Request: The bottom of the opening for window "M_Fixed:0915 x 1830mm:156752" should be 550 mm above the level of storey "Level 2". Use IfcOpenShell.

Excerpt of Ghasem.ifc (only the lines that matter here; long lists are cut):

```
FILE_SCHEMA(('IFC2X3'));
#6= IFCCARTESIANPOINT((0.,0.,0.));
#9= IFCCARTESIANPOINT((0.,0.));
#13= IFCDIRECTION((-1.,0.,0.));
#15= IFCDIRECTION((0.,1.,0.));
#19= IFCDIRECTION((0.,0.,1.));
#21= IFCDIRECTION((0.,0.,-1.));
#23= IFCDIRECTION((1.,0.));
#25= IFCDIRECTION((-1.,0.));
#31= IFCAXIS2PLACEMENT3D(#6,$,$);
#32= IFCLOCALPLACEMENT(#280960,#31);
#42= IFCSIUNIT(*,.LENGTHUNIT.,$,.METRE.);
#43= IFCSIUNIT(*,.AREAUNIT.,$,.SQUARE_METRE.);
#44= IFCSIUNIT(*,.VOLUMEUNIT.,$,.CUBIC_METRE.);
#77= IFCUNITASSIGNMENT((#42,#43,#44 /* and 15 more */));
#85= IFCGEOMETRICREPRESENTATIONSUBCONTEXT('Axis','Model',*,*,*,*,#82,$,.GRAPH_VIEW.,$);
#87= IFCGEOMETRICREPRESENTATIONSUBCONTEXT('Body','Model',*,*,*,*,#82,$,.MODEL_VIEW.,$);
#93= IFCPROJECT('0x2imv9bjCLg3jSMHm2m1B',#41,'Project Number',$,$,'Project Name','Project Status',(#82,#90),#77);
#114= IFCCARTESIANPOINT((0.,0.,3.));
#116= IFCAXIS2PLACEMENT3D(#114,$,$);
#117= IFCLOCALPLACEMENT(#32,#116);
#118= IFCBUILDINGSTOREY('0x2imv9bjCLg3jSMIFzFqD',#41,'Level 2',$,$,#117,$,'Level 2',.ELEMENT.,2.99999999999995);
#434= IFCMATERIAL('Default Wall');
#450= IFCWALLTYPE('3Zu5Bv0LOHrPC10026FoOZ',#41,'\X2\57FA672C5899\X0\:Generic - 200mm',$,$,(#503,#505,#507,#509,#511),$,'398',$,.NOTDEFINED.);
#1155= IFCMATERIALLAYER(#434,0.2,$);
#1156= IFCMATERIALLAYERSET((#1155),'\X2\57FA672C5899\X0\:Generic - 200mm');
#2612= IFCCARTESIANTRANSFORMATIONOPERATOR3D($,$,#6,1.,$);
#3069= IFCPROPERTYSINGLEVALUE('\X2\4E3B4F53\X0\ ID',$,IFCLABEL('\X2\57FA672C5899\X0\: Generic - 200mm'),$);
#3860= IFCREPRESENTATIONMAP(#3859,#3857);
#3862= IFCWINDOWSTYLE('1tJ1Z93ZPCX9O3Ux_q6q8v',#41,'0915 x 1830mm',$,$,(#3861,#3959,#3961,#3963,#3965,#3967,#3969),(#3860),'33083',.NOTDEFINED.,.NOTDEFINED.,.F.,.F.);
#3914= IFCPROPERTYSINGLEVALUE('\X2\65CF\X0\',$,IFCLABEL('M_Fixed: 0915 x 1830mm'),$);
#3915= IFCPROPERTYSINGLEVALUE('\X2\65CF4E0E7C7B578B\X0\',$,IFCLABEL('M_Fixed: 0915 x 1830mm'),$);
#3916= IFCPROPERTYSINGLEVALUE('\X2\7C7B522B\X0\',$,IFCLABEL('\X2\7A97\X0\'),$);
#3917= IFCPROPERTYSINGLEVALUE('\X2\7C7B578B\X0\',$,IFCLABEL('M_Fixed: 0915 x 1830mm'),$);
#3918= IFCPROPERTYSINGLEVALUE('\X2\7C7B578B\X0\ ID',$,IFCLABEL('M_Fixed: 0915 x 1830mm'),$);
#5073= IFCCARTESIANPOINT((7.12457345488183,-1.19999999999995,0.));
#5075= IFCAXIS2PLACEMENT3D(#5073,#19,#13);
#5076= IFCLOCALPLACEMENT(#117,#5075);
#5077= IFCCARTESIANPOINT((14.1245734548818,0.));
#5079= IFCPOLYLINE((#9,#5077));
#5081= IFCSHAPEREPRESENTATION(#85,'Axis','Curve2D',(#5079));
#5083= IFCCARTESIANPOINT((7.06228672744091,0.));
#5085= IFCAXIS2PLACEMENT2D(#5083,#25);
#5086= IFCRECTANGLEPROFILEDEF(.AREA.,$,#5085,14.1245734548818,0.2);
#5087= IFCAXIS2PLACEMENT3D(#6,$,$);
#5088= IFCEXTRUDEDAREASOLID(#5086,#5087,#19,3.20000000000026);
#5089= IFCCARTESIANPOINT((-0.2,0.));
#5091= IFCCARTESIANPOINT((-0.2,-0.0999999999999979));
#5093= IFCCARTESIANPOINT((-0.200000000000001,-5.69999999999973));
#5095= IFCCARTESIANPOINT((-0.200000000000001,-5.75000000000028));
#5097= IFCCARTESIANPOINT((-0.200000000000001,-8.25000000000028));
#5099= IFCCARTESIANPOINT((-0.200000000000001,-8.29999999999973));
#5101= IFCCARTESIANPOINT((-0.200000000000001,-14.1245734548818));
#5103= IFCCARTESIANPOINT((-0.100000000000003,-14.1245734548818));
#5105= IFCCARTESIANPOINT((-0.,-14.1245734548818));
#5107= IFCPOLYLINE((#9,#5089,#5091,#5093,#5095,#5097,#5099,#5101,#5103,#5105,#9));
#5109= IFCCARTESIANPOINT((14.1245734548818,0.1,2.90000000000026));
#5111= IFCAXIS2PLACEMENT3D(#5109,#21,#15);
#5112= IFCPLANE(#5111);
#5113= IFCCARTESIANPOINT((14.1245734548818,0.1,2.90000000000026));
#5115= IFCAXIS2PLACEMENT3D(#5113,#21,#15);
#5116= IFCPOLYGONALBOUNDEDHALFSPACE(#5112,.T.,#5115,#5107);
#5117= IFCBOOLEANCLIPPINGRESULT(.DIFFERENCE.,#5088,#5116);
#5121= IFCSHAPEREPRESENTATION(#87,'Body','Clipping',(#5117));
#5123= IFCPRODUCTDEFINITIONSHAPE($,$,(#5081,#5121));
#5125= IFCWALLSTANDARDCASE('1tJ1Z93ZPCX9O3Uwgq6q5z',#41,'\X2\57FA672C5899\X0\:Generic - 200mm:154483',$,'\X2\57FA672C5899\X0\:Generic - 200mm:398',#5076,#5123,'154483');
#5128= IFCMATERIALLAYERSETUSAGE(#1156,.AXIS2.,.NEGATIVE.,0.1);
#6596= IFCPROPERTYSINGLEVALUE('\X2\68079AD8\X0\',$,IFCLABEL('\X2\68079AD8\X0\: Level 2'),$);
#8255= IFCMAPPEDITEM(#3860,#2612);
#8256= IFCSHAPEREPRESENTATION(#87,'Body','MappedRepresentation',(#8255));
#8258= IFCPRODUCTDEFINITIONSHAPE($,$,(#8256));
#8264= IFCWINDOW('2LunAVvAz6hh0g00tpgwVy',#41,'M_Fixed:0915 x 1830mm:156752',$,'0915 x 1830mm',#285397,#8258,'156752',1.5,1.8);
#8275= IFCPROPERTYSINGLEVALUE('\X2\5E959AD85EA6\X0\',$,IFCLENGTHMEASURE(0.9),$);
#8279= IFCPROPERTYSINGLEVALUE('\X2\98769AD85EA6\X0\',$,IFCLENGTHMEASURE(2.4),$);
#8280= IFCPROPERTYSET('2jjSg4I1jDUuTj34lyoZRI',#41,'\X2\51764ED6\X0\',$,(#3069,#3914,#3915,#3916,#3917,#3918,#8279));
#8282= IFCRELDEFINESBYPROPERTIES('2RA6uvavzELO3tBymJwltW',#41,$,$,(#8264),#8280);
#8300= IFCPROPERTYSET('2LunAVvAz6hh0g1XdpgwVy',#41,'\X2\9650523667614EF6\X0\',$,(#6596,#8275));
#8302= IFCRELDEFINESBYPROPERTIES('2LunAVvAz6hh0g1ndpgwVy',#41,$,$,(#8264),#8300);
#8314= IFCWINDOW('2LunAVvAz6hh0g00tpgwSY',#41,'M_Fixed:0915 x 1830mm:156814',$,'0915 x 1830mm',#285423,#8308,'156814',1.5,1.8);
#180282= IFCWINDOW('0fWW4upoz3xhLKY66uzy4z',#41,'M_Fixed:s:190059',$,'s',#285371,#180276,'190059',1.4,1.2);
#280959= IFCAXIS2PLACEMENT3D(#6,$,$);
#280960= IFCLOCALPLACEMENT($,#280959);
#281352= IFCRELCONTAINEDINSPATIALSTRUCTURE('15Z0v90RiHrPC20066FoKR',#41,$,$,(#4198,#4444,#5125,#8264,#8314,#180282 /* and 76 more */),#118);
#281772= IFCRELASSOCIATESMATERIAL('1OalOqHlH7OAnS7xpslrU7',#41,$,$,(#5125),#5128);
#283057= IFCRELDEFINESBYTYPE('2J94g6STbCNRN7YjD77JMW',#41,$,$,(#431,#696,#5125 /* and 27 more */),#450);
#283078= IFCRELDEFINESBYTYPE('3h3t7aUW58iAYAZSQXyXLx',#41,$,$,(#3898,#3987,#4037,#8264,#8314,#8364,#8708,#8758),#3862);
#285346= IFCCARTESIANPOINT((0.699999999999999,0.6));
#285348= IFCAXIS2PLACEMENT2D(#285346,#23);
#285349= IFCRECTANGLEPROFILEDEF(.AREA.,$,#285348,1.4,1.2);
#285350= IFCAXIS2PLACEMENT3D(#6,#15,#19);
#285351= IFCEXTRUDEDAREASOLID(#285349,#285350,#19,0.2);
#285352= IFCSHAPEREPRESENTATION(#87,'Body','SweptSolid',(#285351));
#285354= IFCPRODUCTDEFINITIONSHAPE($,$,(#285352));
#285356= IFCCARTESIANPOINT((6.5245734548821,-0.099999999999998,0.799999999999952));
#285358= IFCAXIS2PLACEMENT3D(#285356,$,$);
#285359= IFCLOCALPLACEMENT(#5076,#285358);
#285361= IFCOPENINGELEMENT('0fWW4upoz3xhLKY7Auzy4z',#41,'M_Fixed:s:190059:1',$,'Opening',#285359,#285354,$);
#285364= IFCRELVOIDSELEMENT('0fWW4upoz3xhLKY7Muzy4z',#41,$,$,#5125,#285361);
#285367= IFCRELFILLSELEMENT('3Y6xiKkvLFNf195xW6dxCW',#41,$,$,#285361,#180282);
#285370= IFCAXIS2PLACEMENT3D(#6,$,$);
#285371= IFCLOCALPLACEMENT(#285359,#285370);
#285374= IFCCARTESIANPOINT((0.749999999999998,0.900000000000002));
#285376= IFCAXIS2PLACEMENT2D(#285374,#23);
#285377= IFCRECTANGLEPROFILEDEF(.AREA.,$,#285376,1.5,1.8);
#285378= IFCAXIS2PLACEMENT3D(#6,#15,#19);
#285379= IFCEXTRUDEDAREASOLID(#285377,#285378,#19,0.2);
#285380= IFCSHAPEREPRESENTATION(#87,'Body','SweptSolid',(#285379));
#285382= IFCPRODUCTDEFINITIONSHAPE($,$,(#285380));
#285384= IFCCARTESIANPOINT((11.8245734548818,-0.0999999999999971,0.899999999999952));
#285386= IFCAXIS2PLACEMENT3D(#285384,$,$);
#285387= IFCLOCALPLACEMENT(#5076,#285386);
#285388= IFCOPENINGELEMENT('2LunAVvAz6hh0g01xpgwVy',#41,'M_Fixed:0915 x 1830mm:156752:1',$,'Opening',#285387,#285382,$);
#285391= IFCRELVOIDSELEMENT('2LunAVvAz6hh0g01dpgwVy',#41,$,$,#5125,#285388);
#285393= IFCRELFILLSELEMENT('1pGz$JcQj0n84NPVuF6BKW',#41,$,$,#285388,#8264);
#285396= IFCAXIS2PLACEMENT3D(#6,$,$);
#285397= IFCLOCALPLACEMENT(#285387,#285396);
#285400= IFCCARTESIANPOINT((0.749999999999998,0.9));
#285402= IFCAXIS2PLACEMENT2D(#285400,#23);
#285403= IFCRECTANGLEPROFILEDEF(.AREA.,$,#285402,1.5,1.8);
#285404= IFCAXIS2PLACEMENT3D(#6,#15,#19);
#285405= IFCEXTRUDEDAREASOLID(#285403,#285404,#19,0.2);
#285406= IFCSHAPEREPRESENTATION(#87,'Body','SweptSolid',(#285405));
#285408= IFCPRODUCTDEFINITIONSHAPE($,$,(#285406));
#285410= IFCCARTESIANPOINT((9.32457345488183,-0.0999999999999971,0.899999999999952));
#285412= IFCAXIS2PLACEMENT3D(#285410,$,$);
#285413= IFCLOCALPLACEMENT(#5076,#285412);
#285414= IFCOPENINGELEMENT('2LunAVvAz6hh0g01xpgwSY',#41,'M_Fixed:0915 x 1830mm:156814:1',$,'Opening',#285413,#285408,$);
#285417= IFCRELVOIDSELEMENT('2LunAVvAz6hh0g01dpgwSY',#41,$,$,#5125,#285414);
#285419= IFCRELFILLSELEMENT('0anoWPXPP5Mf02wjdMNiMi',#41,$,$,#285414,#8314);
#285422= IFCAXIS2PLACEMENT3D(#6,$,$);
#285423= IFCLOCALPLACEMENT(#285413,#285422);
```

```python
import numpy as np
import ifcopenshell
import ifcopenshell.api.geometry
import ifcopenshell.api.pset
import ifcopenshell.geom
import ifcopenshell.util.element
import ifcopenshell.util.placement
import ifcopenshell.util.shape
import ifcopenshell.util.unit

model = ifcopenshell.open("Ghasem.ifc")
unit_scale = ifcopenshell.util.unit.calculate_unit_scale(model)

window = model.by_id(8264)
opening = window.FillsVoids[0].RelatingOpeningElement
storey = ifcopenshell.util.element.get_container(window, ifc_class="IfcBuildingStorey")
level = ifcopenshell.util.placement.get_local_placement(storey.ObjectPlacement)[2, 3]

# The opening's origin need not be at the sill, so measure its lowest point.
shape = ifcopenshell.geom.create_shape(ifcopenshell.geom.settings(), opening)
bottom = ifcopenshell.util.shape.get_shape_bottom_elevation(shape, shape.geometry) / unit_scale
dz = level + 0.55 - bottom

shift = np.array([0.0, 0.0, dz])
# The window is placed relative to its opening, so it follows when the opening moves.
matrix = ifcopenshell.util.placement.get_local_placement(opening.ObjectPlacement)
matrix[:3, 3] += shift
ifcopenshell.api.geometry.edit_object_placement(
    model, product=opening, matrix=matrix, is_si=False, should_transform_children=True
)

# Keep the stored heights in step.
pset = model.by_id(ifcopenshell.util.element.get_pset(window, "其他", should_inherit=False)["id"])
ifcopenshell.api.pset.edit_pset(model, pset=pset, properties={
    "顶高度": model.create_entity("IfcLengthMeasure", ifcopenshell.util.element.get_pset(window, "其他", "顶高度") + dz),
})
pset = model.by_id(ifcopenshell.util.element.get_pset(window, "限制条件", should_inherit=False)["id"])
ifcopenshell.api.pset.edit_pset(model, pset=pset, properties={
    "底高度": model.create_entity("IfcLengthMeasure", ifcopenshell.util.element.get_pset(window, "限制条件", "底高度") + dz),
})

print(f"moved by {dz * unit_scale:+.3f} m")

model.write("Ghasem_rev.ifc")
```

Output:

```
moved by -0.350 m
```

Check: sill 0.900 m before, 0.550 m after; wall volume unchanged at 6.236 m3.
